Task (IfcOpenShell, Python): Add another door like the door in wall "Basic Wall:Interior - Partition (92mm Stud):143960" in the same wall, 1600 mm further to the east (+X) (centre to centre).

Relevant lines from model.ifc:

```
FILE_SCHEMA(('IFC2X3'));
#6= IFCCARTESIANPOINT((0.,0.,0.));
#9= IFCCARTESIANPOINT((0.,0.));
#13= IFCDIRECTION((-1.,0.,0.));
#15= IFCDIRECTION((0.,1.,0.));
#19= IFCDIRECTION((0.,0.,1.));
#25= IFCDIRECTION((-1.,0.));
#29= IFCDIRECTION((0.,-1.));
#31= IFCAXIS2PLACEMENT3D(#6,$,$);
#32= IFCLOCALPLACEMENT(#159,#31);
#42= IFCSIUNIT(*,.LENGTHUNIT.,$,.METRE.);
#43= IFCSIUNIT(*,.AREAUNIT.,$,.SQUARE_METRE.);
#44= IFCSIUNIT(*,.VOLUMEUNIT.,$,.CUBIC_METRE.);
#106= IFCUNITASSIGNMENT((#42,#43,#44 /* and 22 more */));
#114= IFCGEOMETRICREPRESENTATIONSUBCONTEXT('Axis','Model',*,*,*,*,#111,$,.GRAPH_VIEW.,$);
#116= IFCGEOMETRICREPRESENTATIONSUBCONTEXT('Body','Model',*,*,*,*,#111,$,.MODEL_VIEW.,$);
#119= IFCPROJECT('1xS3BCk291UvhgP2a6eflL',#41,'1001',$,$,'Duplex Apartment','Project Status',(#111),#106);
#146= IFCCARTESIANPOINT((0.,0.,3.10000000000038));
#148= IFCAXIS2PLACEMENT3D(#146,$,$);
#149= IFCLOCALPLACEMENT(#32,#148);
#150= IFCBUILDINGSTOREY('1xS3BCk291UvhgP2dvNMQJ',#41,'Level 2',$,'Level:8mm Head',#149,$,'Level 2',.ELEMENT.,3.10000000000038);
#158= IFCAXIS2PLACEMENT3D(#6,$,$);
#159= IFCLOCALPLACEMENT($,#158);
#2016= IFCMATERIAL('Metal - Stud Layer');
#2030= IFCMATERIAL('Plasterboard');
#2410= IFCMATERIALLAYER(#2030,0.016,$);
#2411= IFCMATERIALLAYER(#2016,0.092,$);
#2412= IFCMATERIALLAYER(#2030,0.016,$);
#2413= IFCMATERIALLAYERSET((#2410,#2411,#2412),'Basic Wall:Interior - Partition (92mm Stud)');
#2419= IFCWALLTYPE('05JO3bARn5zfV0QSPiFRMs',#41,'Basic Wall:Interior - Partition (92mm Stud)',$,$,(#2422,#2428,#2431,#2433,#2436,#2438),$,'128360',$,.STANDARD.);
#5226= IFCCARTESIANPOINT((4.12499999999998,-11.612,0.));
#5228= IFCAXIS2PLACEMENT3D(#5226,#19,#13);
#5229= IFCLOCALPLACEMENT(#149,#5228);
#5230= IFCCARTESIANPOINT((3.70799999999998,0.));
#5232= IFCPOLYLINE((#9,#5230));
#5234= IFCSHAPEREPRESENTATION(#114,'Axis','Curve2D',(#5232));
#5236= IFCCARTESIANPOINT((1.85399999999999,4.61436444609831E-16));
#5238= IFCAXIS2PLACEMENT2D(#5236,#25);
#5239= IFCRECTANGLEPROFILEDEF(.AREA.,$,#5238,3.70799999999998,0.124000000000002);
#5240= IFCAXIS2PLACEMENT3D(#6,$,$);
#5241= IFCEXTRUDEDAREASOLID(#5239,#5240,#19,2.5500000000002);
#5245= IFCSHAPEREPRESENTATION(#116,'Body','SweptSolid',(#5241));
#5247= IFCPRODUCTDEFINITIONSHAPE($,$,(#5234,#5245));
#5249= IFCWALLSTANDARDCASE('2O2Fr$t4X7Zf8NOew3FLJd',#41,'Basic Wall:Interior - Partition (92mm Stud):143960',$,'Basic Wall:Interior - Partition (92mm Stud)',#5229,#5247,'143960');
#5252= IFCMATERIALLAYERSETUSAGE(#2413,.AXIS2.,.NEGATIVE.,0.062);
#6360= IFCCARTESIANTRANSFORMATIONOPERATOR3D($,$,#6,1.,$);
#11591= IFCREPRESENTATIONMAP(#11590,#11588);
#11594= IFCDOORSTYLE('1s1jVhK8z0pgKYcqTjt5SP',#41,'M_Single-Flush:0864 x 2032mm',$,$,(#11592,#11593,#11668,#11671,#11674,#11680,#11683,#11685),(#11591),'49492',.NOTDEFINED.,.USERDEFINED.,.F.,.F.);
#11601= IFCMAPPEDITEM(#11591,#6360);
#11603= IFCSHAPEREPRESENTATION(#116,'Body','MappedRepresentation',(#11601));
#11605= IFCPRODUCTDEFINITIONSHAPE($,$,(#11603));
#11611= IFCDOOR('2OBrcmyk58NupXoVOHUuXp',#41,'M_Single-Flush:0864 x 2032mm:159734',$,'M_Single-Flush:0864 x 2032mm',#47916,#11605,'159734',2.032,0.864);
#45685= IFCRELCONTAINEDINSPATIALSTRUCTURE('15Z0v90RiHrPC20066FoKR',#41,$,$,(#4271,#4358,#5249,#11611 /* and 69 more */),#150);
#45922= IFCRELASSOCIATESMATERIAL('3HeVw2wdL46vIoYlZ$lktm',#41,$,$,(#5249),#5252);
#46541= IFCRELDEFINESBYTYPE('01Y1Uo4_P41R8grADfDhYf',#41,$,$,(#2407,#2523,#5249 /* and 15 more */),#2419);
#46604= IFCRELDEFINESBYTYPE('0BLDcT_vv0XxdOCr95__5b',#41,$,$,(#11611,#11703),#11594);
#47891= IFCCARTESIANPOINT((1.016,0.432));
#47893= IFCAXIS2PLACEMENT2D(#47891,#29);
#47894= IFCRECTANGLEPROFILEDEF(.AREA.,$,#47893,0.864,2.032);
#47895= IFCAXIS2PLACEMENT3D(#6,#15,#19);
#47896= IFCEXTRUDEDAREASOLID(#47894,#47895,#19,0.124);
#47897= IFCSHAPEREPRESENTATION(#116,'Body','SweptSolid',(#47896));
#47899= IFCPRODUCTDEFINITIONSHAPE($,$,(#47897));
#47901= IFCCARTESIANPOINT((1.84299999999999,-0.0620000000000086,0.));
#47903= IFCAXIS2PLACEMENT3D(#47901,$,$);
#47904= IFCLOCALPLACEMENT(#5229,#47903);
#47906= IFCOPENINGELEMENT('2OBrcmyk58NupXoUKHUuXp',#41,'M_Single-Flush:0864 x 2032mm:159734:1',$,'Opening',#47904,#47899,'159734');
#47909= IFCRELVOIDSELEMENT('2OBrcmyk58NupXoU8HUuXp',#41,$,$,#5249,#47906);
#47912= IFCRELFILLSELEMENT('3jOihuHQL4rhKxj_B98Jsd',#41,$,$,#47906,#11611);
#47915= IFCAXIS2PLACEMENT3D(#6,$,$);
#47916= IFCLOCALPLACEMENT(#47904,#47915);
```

```python
import ifcopenshell
import ifcopenshell.api.feature
import ifcopenshell.api.geometry
import ifcopenshell.api.root
import ifcopenshell.geom
import ifcopenshell.util.element
import ifcopenshell.util.placement
import ifcopenshell.util.shape
import ifcopenshell.util.unit

model = ifcopenshell.open("model.ifc")
unit_scale = ifcopenshell.util.unit.calculate_unit_scale(model)
settings = ifcopenshell.geom.settings()


def volume(element):
    """Net volume in cubic metres, openings subtracted."""
    shape = ifcopenshell.geom.create_shape(settings, element)
    return ifcopenshell.util.shape.get_volume(shape.geometry)


def reuse_history(source, copy):
    """copy_class also copies each property set's owner history, people and application; keep the originals."""
    for rel in copy.IsDefinedBy:
        if rel.is_a("IfcRelDefinesByProperties") and (history := rel.RelatingPropertyDefinition.OwnerHistory):
            rel.RelatingPropertyDefinition.OwnerHistory = source.OwnerHistory
            ifcopenshell.util.element.remove_deep2(model, history)


door = model.by_guid("2OBrcmyk58NupXoVOHUuXp")
opening = door.FillsVoids[0].RelatingOpeningElement
wall = opening.VoidsElements[0].RelatingBuildingElement
before = volume(wall)
shift = ifcopenshell.util.placement.get_local_placement(wall.ObjectPlacement)[:3, 0] * -1.6 / unit_scale

# copy_class copies the void relationship, type, container and properties, but no geometry.
new_opening = ifcopenshell.api.root.copy_class(model, product=opening)
new_opening.Representation = ifcopenshell.util.element.copy_deep(
    model, opening.Representation, exclude=["IfcGeometricRepresentationContext", "IfcRepresentationMap"]
)
new_opening.Name = "M_Single-Flush:0864 x 2032mm"
new_opening.Tag = None
new_door = ifcopenshell.api.root.copy_class(model, product=door)
new_door.Representation = ifcopenshell.util.element.copy_deep(
    model, door.Representation, exclude=["IfcGeometricRepresentationContext", "IfcRepresentationMap"]
)
new_door.Name = "M_Single-Flush:0864 x 2032mm"
new_door.Tag = None
reuse_history(door, new_door)
fills = ifcopenshell.api.feature.add_filling(model, opening=new_opening, element=new_door)
fills.OwnerHistory = new_door.OwnerHistory  # required in IFC2X3

for old, new in ((opening, new_opening), (door, new_door)):
    matrix = ifcopenshell.util.placement.get_local_placement(old.ObjectPlacement)
    matrix[:3, 3] += shift
    ifcopenshell.api.geometry.edit_object_placement(model, product=new, matrix=matrix, is_si=False)

after = volume(wall)

print(f"wall volume {before:.3f} -> {after:.3f} m3")

model.write("model_edited.ifc")
```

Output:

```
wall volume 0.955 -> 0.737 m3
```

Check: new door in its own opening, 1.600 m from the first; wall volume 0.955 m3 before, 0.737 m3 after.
